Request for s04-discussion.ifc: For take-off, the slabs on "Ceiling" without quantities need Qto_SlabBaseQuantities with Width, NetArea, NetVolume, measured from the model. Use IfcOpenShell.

First a look at what the model holds.

```python
import ifcopenshell
import ifcopenshell.util.element
import ifcopenshell.util.unit

model = ifcopenshell.open("s04-discussion.ifc")
print(model.schema)
for unit_type in ("LENGTHUNIT", "AREAUNIT", "VOLUMEUNIT"):
    print(unit_type, ifcopenshell.util.unit.calculate_unit_scale(model, unit_type))
storey = next(s for s in model.by_type("IfcBuildingStorey") if s.Name == "Ceiling")
slabs = [e for e in ifcopenshell.util.element.get_decomposition(storey) if e.is_a("IfcSlab")]
for e in sorted(slabs, key=lambda e: e.id()):
    print(e.id(), e.is_a(), e.Name, list(ifcopenshell.util.element.get_psets(e, qtos_only=True)), sep=" | ")
```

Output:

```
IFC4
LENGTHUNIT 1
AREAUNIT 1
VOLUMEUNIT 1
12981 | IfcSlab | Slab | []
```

```python
import ifcopenshell
import ifcopenshell.api.pset
import ifcopenshell.geom
import ifcopenshell.util.element
import ifcopenshell.util.shape
import ifcopenshell.util.unit

model = ifcopenshell.open("s04-discussion.ifc")
unit_scale = ifcopenshell.util.unit.calculate_unit_scale(model)
area_scale = ifcopenshell.util.unit.calculate_unit_scale(model, "AREAUNIT")
volume_scale = ifcopenshell.util.unit.calculate_unit_scale(model, "VOLUMEUNIT")
settings = ifcopenshell.geom.settings()

storey = next(s for s in model.by_type("IfcBuildingStorey") if s.Name == "Ceiling")
slabs = [e for e in ifcopenshell.util.element.get_decomposition(storey) if e.is_a("IfcSlab")]

for e in sorted(slabs, key=lambda e: e.id()):
    if ifcopenshell.util.element.get_psets(e, qtos_only=True, should_inherit=False):
        continue
    # Geometry comes back in metres, in the element's own axes.
    shape = ifcopenshell.geom.create_shape(settings, e)
    values = {
        "Width": ifcopenshell.util.shape.get_z(shape.geometry) / unit_scale,
        "NetArea": ifcopenshell.util.shape.get_footprint_area(shape.geometry) / area_scale,
        "NetVolume": ifcopenshell.util.shape.get_volume(shape.geometry) / volume_scale,
    }
    qto = ifcopenshell.api.pset.add_qto(model, product=e, name="Qto_SlabBaseQuantities")
    ifcopenshell.api.pset.edit_qto(model, qto=qto, properties=values)
    print(e.id(), {k: round(v, 3) for k, v in values.items()})

model.write("s04-discussion_edited.ifc")
```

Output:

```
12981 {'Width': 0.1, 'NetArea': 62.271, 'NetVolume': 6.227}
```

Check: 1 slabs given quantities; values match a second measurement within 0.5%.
